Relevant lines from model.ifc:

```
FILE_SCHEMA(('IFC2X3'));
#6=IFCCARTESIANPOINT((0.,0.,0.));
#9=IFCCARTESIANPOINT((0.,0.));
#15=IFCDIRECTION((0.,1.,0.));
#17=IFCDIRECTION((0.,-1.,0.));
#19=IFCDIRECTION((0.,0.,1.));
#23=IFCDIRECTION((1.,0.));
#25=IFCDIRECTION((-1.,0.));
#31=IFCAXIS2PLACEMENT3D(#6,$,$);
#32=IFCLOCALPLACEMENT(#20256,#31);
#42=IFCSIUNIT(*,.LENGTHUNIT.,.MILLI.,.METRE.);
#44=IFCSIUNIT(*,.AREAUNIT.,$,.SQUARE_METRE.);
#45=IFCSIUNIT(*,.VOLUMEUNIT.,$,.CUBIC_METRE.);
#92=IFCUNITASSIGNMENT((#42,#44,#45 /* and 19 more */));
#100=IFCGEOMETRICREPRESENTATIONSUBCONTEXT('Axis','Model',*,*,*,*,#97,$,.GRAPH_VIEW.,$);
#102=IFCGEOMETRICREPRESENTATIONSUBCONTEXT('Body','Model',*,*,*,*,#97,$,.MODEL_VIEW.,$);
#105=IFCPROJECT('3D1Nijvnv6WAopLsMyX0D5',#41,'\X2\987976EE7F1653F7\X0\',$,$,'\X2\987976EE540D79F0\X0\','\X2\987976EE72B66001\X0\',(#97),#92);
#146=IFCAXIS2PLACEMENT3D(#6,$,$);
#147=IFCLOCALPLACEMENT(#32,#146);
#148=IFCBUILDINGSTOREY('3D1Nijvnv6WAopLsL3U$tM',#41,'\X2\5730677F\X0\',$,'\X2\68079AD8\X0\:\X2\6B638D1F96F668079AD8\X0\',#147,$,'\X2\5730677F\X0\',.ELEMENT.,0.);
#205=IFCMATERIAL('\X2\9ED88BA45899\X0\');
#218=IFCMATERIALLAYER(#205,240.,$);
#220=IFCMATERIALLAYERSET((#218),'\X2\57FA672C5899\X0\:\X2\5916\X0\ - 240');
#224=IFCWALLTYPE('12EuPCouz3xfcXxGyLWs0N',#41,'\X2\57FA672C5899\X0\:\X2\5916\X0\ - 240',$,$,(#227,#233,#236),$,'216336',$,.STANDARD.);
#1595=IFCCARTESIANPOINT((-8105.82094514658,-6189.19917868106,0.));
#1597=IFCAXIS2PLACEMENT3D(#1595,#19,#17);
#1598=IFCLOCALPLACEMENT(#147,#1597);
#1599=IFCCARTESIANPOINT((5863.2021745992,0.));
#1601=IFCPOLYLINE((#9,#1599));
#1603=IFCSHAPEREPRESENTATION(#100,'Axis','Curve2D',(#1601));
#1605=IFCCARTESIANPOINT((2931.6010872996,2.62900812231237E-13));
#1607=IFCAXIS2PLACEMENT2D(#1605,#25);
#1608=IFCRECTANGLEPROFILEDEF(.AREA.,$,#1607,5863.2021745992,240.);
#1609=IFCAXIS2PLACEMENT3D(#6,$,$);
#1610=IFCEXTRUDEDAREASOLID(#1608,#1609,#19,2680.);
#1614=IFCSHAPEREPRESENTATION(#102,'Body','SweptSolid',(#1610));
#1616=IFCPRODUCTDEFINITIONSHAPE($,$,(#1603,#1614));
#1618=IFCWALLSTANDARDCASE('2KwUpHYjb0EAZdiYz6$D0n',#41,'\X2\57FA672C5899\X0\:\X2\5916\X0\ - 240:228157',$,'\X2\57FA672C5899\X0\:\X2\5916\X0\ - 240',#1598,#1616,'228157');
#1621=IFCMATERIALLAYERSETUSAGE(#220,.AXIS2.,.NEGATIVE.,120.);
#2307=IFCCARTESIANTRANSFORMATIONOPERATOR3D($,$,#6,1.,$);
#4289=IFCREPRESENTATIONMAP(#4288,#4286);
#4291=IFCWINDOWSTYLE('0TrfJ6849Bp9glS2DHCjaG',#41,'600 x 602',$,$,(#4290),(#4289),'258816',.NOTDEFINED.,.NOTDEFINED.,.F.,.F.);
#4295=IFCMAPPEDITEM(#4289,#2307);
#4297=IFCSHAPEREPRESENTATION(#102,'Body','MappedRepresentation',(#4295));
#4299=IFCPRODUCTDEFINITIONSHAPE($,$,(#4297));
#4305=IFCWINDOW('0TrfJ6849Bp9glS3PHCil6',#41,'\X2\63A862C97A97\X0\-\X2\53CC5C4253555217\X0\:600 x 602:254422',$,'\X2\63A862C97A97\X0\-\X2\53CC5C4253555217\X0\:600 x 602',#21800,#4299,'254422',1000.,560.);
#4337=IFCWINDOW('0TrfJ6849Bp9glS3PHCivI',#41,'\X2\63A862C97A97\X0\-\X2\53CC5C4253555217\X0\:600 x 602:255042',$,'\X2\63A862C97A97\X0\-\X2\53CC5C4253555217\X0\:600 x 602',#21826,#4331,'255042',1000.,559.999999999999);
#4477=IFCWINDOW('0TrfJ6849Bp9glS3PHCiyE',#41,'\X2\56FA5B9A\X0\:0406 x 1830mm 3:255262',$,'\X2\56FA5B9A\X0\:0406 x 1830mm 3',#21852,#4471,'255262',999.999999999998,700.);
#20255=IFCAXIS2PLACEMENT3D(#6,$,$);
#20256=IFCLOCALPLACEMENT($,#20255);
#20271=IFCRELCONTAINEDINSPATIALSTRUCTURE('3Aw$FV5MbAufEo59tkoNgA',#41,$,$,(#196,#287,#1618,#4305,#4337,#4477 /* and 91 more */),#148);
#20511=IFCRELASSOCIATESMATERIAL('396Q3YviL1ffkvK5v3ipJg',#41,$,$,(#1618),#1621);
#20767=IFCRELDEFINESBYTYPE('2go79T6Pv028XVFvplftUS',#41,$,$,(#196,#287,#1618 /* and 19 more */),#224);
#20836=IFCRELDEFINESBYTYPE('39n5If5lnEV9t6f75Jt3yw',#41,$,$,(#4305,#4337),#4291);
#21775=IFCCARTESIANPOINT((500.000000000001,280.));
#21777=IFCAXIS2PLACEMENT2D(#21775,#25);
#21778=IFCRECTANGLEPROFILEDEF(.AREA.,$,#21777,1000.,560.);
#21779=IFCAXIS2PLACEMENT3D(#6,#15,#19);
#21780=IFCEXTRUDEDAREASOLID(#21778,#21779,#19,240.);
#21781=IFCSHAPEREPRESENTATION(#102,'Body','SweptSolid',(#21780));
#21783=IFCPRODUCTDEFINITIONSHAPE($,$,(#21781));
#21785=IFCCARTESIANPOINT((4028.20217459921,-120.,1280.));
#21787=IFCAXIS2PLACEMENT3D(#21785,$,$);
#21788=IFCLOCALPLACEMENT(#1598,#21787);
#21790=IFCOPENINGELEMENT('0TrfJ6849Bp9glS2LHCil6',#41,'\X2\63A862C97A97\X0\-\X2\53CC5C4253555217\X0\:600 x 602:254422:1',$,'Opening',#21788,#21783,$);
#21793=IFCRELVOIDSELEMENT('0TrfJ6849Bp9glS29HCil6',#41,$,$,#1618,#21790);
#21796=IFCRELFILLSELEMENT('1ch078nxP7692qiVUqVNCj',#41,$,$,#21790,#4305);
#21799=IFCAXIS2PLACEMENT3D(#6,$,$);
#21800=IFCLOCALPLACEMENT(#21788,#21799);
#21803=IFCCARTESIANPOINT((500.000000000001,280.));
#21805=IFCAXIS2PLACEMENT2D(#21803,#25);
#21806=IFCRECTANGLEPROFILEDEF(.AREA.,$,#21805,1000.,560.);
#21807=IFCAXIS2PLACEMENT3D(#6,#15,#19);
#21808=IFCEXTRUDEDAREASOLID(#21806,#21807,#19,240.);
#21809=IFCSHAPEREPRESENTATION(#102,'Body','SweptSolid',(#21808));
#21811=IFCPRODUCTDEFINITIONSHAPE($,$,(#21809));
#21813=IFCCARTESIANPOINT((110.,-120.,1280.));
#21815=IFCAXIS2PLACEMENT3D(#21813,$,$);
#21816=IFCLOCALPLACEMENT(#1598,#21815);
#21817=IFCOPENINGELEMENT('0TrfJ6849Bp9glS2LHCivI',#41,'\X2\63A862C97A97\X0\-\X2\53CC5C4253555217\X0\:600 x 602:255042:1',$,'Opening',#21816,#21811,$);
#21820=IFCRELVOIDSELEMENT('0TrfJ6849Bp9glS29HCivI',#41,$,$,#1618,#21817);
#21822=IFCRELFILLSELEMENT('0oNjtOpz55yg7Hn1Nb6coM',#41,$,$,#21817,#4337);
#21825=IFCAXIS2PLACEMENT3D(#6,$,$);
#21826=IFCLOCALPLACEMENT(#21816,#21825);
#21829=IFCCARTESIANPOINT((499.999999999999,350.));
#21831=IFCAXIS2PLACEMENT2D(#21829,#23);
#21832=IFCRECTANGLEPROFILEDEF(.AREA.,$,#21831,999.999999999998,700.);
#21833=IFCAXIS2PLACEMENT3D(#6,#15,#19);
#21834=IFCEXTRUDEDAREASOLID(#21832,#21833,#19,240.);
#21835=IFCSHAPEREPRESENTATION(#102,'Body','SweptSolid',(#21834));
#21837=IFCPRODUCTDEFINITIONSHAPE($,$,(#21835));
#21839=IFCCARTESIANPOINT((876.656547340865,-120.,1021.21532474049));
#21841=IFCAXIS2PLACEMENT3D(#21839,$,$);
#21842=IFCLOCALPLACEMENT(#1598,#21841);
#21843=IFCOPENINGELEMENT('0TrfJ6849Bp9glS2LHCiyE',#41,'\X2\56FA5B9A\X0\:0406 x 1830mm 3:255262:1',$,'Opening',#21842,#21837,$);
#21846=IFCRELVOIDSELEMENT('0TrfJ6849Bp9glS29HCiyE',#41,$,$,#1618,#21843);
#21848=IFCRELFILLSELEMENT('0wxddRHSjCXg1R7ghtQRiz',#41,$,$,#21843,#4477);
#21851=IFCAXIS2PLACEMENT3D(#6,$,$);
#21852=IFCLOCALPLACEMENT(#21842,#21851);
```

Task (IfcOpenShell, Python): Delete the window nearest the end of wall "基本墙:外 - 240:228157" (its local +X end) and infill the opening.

```python
import ifcopenshell
import ifcopenshell.api.feature
import ifcopenshell.api.root
import ifcopenshell.geom
import ifcopenshell.util.shape

model = ifcopenshell.open("model.ifc")
settings = ifcopenshell.geom.settings()


def volume(element):
    """Net volume in cubic metres, openings subtracted."""
    shape = ifcopenshell.geom.create_shape(settings, element)
    return ifcopenshell.util.shape.get_volume(shape.geometry)


window = model.by_guid("0TrfJ6849Bp9glS3PHCil6")
opening = window.FillsVoids[0].RelatingOpeningElement
wall = opening.VoidsElements[0].RelatingBuildingElement
before = volume(wall)

ifcopenshell.api.root.remove_product(model, product=window)
ifcopenshell.api.feature.remove_feature(model, feature=opening)

after = volume(wall)

print(f"wall volume {before:.3f} -> {after:.3f} m3")

model.write("model_edited.ifc")
```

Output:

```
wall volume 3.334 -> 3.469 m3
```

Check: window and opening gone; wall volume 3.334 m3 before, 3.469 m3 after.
